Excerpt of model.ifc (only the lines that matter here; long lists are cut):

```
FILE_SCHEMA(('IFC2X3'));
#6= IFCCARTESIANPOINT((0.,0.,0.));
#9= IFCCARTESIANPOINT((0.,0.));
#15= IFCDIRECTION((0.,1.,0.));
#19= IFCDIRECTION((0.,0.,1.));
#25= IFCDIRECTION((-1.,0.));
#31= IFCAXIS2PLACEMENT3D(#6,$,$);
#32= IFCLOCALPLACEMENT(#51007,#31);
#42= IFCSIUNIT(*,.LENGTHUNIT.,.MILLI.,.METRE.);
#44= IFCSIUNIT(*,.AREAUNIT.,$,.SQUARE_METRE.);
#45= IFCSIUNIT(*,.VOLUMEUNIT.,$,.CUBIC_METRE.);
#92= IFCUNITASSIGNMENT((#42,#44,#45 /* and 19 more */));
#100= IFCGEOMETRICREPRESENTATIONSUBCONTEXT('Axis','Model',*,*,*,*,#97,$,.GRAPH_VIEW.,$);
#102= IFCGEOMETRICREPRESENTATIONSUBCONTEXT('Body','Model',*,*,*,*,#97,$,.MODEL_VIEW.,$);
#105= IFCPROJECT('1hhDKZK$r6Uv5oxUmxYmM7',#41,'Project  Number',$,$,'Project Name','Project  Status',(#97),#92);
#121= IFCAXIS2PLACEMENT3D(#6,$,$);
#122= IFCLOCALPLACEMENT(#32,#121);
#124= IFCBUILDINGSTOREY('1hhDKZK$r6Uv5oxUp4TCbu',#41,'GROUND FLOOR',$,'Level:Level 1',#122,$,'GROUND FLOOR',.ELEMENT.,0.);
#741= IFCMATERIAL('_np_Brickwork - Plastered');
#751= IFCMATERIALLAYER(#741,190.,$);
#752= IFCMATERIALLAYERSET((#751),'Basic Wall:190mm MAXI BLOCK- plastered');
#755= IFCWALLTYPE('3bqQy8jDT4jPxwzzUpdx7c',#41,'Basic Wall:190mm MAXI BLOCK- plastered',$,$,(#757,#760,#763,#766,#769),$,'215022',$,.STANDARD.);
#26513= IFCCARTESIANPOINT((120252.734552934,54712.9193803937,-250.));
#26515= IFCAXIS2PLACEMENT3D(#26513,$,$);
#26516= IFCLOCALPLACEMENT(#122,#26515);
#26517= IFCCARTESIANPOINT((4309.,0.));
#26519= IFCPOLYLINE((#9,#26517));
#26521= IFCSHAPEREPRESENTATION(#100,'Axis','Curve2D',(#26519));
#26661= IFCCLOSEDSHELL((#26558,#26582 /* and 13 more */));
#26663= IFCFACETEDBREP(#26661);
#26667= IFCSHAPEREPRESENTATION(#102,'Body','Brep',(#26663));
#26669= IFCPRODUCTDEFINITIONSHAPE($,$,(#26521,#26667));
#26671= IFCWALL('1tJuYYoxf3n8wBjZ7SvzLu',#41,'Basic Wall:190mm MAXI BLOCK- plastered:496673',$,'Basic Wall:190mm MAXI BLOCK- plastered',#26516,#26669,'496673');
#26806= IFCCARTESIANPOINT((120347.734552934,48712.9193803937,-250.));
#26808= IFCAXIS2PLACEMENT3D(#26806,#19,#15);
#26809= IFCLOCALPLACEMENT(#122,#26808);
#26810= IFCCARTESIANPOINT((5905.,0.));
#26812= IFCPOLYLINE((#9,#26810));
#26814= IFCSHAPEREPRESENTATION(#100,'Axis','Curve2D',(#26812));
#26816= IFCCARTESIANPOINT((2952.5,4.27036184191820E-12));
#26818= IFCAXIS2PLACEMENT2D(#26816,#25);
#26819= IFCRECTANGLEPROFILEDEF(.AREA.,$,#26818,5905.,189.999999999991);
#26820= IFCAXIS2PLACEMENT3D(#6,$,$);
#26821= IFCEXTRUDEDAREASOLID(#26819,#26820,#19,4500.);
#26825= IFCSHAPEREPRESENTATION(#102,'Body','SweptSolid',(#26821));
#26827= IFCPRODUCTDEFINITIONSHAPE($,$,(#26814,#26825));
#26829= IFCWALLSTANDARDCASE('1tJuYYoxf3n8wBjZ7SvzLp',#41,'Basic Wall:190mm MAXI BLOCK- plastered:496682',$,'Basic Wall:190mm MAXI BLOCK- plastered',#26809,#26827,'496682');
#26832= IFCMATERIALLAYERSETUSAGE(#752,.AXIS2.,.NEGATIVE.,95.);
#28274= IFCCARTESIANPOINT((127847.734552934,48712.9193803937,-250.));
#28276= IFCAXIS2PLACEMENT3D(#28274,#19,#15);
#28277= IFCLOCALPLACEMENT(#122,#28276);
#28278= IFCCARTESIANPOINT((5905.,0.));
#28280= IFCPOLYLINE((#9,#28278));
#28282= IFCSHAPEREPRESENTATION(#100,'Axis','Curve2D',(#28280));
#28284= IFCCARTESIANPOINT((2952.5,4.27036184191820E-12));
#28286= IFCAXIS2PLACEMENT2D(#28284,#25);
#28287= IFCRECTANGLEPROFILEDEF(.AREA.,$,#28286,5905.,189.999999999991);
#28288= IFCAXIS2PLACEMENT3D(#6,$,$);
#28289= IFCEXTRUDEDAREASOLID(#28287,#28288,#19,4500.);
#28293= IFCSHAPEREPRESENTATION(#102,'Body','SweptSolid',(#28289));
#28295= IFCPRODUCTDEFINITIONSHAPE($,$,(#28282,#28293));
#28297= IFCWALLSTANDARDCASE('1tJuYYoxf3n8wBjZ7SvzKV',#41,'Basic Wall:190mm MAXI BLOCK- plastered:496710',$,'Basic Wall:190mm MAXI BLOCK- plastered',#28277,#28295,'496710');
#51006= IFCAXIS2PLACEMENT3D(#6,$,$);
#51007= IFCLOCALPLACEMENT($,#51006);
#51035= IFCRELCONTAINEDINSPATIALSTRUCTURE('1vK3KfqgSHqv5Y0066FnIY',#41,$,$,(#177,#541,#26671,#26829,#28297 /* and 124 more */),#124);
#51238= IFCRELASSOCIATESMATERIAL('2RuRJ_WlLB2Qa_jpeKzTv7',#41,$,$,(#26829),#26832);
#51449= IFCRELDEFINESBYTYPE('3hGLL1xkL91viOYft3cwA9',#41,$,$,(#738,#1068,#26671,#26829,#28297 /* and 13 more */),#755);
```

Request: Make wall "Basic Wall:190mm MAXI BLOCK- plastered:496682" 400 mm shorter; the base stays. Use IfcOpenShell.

```python
import ifcopenshell
import ifcopenshell.geom
import ifcopenshell.util.representation
import ifcopenshell.util.shape
import ifcopenshell.util.unit

model = ifcopenshell.open("model.ifc")
unit_scale = ifcopenshell.util.unit.calculate_unit_scale(model)
settings = ifcopenshell.geom.settings()


def volume(element):
    """Net volume in cubic metres, openings subtracted."""
    shape = ifcopenshell.geom.create_shape(settings, element)
    return ifcopenshell.util.shape.get_volume(shape.geometry)


wall = model.by_id(26829)
before = volume(wall)

body = ifcopenshell.util.representation.get_representation(wall, "Model", "Body")
solid = body.Items[0]
old_height = solid.Depth
solid.Depth -= 0.4 / unit_scale
after = volume(wall)

print(f"height {old_height:g} -> {solid.Depth:g}, volume {before:.3f} -> {after:.3f} m3")

model.write("model_updated.ifc")
```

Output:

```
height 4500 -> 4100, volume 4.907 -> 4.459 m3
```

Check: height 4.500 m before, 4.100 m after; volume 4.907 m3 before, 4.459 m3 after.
